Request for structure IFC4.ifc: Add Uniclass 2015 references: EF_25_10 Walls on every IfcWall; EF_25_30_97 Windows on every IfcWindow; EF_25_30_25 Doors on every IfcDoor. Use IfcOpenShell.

First a look at what the model holds.

```python
import ifcopenshell

model = ifcopenshell.open("structure IFC4.ifc")
print(model.schema)
print("classifications:", [c.Name for c in model.by_type("IfcClassification")])
for ifc_class in ("IfcDoor", "IfcRoof", "IfcStair", "IfcWall", "IfcWindow"):
    print(ifc_class, len(model.by_type(ifc_class)))
```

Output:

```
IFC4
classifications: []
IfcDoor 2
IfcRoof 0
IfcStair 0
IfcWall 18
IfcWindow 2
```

```python
import ifcopenshell
import ifcopenshell.api.classification

model = ifcopenshell.open("structure IFC4.ifc")

system = ifcopenshell.api.classification.add_classification(model, classification="Uniclass 2015")

codes = {
    "IfcWall": ("EF_25_10", "Walls"),
    "IfcWindow": ("EF_25_30_97", "Windows"),
    "IfcDoor": ("EF_25_30_25", "Doors"),
}
for ifc_class, (code, name) in codes.items():
    products = model.by_type(ifc_class)
    ifcopenshell.api.classification.add_reference(
        model, products=products, classification=system, identification=code, name=name
    )
    print(code, len(products))

model.write("structure IFC4-out.ifc")
```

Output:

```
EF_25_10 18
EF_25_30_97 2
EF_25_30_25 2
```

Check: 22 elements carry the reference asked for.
